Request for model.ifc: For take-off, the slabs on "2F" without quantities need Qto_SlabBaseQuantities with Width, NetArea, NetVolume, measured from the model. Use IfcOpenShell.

First a look at what the model holds.

```python
import ifcopenshell
import ifcopenshell.util.element
import ifcopenshell.util.unit

model = ifcopenshell.open("model.ifc")
print(model.schema)
for unit_type in ("LENGTHUNIT", "AREAUNIT", "VOLUMEUNIT"):
    print(unit_type, ifcopenshell.util.unit.calculate_unit_scale(model, unit_type))
storey = next(s for s in model.by_type("IfcBuildingStorey") if s.Name == "2F")
slabs = [e for e in ifcopenshell.util.element.get_decomposition(storey) if e.is_a("IfcSlab")]
for e in sorted(slabs, key=lambda e: e.id()):
    print(e.id(), e.is_a(), e.Name, list(ifcopenshell.util.element.get_psets(e, qtos_only=True)), sep=" | ")
```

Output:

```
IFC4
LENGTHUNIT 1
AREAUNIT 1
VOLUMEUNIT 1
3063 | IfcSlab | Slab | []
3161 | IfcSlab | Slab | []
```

```python
import ifcopenshell
import ifcopenshell.api.pset
import ifcopenshell.geom
import ifcopenshell.util.element
import ifcopenshell.util.shape
import ifcopenshell.util.unit

model = ifcopenshell.open("model.ifc")
unit_scale = ifcopenshell.util.unit.calculate_unit_scale(model)
area_scale = ifcopenshell.util.unit.calculate_unit_scale(model, "AREAUNIT")
volume_scale = ifcopenshell.util.unit.calculate_unit_scale(model, "VOLUMEUNIT")
settings = ifcopenshell.geom.settings()

storey = next(s for s in model.by_type("IfcBuildingStorey") if s.Name == "2F")
slabs = [e for e in ifcopenshell.util.element.get_decomposition(storey) if e.is_a("IfcSlab")]

for e in sorted(slabs, key=lambda e: e.id()):
    if ifcopenshell.util.element.get_psets(e, qtos_only=True, should_inherit=False):
        continue
    # Geometry comes back in metres, in the element's own axes.
    shape = ifcopenshell.geom.create_shape(settings, e)
    values = {
        "Width": ifcopenshell.util.shape.get_z(shape.geometry) / unit_scale,
        "NetArea": ifcopenshell.util.shape.get_footprint_area(shape.geometry) / area_scale,
        "NetVolume": ifcopenshell.util.shape.get_volume(shape.geometry) / volume_scale,
    }
    qto = ifcopenshell.api.pset.add_qto(model, product=e, name="Qto_SlabBaseQuantities")
    ifcopenshell.api.pset.edit_qto(model, qto=qto, properties=values)
    print(e.id(), {k: round(v, 3) for k, v in values.items()})

model.write("model_edited.ifc")
```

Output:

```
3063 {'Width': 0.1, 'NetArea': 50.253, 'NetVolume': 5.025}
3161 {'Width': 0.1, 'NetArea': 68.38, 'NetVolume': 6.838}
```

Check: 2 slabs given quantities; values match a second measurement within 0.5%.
